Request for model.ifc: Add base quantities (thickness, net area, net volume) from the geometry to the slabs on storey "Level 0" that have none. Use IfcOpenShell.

First a look at what the model holds.

```python
import ifcopenshell
import ifcopenshell.util.element
import ifcopenshell.util.unit

model = ifcopenshell.open("model.ifc")
print(model.schema)
for unit_type in ("LENGTHUNIT", "AREAUNIT", "VOLUMEUNIT"):
    print(unit_type, ifcopenshell.util.unit.calculate_unit_scale(model, unit_type))
storey = next(s for s in model.by_type("IfcBuildingStorey") if s.Name == "Level 0")
slabs = [e for e in ifcopenshell.util.element.get_decomposition(storey) if e.is_a("IfcSlab")]
for e in sorted(slabs, key=lambda e: e.id()):
    print(e.id(), e.is_a(), e.Name, list(ifcopenshell.util.element.get_psets(e, qtos_only=True)), sep=" | ")
```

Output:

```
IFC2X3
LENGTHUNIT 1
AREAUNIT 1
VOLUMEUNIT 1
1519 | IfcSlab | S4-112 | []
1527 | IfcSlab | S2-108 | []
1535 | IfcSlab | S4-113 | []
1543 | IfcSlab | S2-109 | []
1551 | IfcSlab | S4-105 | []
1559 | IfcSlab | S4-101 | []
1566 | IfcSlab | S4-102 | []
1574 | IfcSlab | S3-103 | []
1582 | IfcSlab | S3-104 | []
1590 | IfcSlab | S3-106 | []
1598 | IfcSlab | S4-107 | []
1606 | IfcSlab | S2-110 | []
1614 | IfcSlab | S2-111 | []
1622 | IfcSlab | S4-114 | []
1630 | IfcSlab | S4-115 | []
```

```python
import ifcopenshell
import ifcopenshell.api.pset
import ifcopenshell.geom
import ifcopenshell.util.element
import ifcopenshell.util.shape
import ifcopenshell.util.unit

model = ifcopenshell.open("model.ifc")
unit_scale = ifcopenshell.util.unit.calculate_unit_scale(model)
area_scale = ifcopenshell.util.unit.calculate_unit_scale(model, "AREAUNIT")
volume_scale = ifcopenshell.util.unit.calculate_unit_scale(model, "VOLUMEUNIT")
settings = ifcopenshell.geom.settings()

storey = next(s for s in model.by_type("IfcBuildingStorey") if s.Name == "Level 0")
slabs = [e for e in ifcopenshell.util.element.get_decomposition(storey) if e.is_a("IfcSlab")]

for e in sorted(slabs, key=lambda e: e.id()):
    if ifcopenshell.util.element.get_psets(e, qtos_only=True, should_inherit=False):
        continue
    # Geometry comes back in metres, in the element's own axes.
    shape = ifcopenshell.geom.create_shape(settings, e)
    values = {
        "Width": ifcopenshell.util.shape.get_z(shape.geometry) / unit_scale,
        "NetArea": ifcopenshell.util.shape.get_footprint_area(shape.geometry) / area_scale,
        "NetVolume": ifcopenshell.util.shape.get_volume(shape.geometry) / volume_scale,
    }
    qto = ifcopenshell.api.pset.add_qto(model, product=e, name="BaseQuantities")
    ifcopenshell.api.pset.edit_qto(model, qto=qto, properties=values)
    print(e.id(), {k: round(v, 3) for k, v in values.items()})

model.write("model-out.ifc")
```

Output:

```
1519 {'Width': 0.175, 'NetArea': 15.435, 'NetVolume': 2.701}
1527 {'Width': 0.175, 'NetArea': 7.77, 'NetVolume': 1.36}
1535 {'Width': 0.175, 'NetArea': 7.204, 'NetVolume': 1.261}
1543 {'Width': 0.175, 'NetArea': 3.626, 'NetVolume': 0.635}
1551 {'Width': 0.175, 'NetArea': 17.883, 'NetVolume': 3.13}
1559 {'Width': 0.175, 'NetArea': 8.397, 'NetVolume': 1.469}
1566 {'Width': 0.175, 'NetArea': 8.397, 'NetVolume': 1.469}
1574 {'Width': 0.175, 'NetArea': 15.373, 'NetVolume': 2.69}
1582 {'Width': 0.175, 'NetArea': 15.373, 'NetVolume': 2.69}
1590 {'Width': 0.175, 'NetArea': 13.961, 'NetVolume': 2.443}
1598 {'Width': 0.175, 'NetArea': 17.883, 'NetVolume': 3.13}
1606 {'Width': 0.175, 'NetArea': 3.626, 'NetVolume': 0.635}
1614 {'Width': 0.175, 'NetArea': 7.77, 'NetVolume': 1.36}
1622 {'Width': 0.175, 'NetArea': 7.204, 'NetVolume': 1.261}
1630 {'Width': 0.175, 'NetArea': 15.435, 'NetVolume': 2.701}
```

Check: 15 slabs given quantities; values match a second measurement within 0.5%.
